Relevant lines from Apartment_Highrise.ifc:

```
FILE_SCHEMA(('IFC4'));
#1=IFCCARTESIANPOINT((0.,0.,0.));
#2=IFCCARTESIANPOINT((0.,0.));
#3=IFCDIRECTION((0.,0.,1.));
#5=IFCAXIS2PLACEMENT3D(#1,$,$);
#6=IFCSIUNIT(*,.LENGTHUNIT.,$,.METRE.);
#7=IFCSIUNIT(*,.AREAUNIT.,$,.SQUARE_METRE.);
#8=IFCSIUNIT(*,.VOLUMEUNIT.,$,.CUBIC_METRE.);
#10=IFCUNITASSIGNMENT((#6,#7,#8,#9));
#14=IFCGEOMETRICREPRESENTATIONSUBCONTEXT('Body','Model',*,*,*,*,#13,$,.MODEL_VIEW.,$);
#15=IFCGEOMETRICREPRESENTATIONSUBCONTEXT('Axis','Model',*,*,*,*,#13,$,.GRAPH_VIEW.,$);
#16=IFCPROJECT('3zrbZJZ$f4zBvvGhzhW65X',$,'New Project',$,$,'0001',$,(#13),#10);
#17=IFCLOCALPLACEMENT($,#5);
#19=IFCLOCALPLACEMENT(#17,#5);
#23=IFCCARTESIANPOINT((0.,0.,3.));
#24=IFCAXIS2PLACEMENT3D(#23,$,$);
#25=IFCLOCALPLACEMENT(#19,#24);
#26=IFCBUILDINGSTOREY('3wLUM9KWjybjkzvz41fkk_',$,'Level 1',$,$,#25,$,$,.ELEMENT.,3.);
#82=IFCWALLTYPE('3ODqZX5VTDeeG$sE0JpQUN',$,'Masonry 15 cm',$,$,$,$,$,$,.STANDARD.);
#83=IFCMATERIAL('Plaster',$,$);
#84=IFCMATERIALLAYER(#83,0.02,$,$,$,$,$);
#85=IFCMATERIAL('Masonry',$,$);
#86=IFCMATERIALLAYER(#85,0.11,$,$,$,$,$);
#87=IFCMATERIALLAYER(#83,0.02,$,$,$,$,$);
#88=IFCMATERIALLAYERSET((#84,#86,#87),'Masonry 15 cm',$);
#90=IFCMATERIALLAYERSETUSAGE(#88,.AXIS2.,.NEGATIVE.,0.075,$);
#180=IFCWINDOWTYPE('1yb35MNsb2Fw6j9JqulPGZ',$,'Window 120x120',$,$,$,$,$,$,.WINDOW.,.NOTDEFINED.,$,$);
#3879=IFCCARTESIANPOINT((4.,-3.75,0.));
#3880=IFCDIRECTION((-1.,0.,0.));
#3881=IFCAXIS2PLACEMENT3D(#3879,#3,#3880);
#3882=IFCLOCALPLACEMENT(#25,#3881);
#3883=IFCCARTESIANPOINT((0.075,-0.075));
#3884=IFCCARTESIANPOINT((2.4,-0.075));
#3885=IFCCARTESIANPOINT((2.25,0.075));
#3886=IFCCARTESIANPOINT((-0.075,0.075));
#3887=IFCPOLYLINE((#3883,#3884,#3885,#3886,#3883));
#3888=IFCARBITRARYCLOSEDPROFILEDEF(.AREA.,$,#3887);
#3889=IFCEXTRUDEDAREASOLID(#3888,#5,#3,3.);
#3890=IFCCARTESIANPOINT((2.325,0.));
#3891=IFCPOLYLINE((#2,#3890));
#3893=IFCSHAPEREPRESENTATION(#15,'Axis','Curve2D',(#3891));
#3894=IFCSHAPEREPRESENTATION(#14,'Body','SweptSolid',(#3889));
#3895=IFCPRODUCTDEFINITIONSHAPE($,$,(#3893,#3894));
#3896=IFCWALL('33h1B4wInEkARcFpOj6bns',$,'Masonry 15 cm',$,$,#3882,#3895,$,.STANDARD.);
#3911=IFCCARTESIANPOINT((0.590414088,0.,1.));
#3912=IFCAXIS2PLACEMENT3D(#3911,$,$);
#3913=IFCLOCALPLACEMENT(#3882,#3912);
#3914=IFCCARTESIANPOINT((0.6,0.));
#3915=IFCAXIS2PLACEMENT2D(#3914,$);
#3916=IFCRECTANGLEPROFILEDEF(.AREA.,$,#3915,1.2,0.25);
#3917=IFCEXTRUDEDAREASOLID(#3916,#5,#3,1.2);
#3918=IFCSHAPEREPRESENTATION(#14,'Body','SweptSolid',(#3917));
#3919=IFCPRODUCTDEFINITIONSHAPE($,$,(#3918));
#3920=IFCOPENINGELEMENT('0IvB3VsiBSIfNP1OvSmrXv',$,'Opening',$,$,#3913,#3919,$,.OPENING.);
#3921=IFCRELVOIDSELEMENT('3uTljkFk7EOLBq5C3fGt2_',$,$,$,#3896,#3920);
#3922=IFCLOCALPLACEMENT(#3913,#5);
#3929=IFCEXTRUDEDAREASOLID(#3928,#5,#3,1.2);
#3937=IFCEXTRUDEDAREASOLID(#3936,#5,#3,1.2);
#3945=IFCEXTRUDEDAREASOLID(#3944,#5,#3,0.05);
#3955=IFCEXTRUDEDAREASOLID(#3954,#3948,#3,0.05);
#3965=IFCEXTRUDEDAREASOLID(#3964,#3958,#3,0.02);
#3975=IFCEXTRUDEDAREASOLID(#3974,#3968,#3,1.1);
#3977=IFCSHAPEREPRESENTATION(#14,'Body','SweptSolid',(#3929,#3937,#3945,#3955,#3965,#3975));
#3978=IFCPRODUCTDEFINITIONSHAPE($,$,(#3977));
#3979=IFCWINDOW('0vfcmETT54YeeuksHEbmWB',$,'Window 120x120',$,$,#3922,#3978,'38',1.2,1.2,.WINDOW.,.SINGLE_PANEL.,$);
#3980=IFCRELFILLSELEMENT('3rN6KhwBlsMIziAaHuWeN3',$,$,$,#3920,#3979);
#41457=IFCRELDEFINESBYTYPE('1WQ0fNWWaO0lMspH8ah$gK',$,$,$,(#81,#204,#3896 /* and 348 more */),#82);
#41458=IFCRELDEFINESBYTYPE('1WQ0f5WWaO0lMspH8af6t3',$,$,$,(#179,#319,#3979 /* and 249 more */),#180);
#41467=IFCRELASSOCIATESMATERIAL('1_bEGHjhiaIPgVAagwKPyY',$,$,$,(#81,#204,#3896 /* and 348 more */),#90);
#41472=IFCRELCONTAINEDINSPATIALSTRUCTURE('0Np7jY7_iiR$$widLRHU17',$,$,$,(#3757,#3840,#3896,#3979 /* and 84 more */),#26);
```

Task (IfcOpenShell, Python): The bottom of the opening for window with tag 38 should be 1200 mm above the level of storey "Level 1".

```python
import numpy as np
import ifcopenshell
import ifcopenshell.api.geometry
import ifcopenshell.geom
import ifcopenshell.util.element
import ifcopenshell.util.placement
import ifcopenshell.util.shape
import ifcopenshell.util.unit

model = ifcopenshell.open("Apartment_Highrise.ifc")
unit_scale = ifcopenshell.util.unit.calculate_unit_scale(model)

window = model.by_guid("0vfcmETT54YeeuksHEbmWB")
opening = window.FillsVoids[0].RelatingOpeningElement
storey = ifcopenshell.util.element.get_container(window, ifc_class="IfcBuildingStorey")
level = ifcopenshell.util.placement.get_local_placement(storey.ObjectPlacement)[2, 3]

# The opening's origin need not be at the sill, so measure its lowest point.
shape = ifcopenshell.geom.create_shape(ifcopenshell.geom.settings(), opening)
bottom = ifcopenshell.util.shape.get_shape_bottom_elevation(shape, shape.geometry) / unit_scale
dz = level + 1.2 / unit_scale - bottom

shift = np.array([0.0, 0.0, dz])
# The window is placed relative to its opening, so it follows when the opening moves.
matrix = ifcopenshell.util.placement.get_local_placement(opening.ObjectPlacement)
matrix[:3, 3] += shift
ifcopenshell.api.geometry.edit_object_placement(
    model, product=opening, matrix=matrix, is_si=False, should_transform_children=True
)

print(f"moved by {dz * unit_scale:+.3f} m")

model.write("Apartment_Highrise-out.ifc")
```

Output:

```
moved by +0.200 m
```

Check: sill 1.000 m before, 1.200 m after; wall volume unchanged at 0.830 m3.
